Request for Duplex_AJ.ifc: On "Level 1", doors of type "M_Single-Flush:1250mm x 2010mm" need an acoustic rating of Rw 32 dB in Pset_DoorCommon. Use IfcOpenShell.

First a look at what the model holds.

```python
import ifcopenshell
import ifcopenshell.util.element

model = ifcopenshell.open("Duplex_AJ.ifc")
print(model.schema)
storey = next(s for s in model.by_type("IfcBuildingStorey") if s.Name == "Level 1")
doors = [e for e in ifcopenshell.util.element.get_decomposition(storey) if e.is_a("IfcDoor")]
seen = {}
for e in doors:
    element_type = ifcopenshell.util.element.get_type(e)
    key = (element_type.Name if element_type != e and element_type else None, ifcopenshell.util.element.get_pset(e, "Pset_DoorCommon", "AcousticRating"))
    seen[key] = seen.get(key, 0) + 1
for (name, value), count in sorted(seen.items(), key=str):
    print(count, "x", name, "|", value)
```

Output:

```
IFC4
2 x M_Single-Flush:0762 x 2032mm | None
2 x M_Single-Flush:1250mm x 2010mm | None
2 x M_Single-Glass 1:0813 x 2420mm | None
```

```python
import ifcopenshell
import ifcopenshell.api.pset
import ifcopenshell.util.element

model = ifcopenshell.open("Duplex_AJ.ifc")

storey = next(s for s in model.by_type("IfcBuildingStorey") if s.Name == "Level 1")
doors = [e for e in ifcopenshell.util.element.get_decomposition(storey) if e.is_a("IfcDoor")]

count = 0
for e in doors:
    element_type = ifcopenshell.util.element.get_type(e)
    if element_type in (None, e) or element_type.Name != "M_Single-Flush:1250mm x 2010mm":
        continue
    # add_pset returns the element's existing set when there is one.
    pset = ifcopenshell.api.pset.add_pset(model, product=e, name="Pset_DoorCommon")
    ifcopenshell.api.pset.edit_pset(model, pset=pset, properties={"AcousticRating": "Rw 32 dB"})
    count += 1

print(count, "doors updated")

model.write("Duplex_AJ_v2.ifc")
```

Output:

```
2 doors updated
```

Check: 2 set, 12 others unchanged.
